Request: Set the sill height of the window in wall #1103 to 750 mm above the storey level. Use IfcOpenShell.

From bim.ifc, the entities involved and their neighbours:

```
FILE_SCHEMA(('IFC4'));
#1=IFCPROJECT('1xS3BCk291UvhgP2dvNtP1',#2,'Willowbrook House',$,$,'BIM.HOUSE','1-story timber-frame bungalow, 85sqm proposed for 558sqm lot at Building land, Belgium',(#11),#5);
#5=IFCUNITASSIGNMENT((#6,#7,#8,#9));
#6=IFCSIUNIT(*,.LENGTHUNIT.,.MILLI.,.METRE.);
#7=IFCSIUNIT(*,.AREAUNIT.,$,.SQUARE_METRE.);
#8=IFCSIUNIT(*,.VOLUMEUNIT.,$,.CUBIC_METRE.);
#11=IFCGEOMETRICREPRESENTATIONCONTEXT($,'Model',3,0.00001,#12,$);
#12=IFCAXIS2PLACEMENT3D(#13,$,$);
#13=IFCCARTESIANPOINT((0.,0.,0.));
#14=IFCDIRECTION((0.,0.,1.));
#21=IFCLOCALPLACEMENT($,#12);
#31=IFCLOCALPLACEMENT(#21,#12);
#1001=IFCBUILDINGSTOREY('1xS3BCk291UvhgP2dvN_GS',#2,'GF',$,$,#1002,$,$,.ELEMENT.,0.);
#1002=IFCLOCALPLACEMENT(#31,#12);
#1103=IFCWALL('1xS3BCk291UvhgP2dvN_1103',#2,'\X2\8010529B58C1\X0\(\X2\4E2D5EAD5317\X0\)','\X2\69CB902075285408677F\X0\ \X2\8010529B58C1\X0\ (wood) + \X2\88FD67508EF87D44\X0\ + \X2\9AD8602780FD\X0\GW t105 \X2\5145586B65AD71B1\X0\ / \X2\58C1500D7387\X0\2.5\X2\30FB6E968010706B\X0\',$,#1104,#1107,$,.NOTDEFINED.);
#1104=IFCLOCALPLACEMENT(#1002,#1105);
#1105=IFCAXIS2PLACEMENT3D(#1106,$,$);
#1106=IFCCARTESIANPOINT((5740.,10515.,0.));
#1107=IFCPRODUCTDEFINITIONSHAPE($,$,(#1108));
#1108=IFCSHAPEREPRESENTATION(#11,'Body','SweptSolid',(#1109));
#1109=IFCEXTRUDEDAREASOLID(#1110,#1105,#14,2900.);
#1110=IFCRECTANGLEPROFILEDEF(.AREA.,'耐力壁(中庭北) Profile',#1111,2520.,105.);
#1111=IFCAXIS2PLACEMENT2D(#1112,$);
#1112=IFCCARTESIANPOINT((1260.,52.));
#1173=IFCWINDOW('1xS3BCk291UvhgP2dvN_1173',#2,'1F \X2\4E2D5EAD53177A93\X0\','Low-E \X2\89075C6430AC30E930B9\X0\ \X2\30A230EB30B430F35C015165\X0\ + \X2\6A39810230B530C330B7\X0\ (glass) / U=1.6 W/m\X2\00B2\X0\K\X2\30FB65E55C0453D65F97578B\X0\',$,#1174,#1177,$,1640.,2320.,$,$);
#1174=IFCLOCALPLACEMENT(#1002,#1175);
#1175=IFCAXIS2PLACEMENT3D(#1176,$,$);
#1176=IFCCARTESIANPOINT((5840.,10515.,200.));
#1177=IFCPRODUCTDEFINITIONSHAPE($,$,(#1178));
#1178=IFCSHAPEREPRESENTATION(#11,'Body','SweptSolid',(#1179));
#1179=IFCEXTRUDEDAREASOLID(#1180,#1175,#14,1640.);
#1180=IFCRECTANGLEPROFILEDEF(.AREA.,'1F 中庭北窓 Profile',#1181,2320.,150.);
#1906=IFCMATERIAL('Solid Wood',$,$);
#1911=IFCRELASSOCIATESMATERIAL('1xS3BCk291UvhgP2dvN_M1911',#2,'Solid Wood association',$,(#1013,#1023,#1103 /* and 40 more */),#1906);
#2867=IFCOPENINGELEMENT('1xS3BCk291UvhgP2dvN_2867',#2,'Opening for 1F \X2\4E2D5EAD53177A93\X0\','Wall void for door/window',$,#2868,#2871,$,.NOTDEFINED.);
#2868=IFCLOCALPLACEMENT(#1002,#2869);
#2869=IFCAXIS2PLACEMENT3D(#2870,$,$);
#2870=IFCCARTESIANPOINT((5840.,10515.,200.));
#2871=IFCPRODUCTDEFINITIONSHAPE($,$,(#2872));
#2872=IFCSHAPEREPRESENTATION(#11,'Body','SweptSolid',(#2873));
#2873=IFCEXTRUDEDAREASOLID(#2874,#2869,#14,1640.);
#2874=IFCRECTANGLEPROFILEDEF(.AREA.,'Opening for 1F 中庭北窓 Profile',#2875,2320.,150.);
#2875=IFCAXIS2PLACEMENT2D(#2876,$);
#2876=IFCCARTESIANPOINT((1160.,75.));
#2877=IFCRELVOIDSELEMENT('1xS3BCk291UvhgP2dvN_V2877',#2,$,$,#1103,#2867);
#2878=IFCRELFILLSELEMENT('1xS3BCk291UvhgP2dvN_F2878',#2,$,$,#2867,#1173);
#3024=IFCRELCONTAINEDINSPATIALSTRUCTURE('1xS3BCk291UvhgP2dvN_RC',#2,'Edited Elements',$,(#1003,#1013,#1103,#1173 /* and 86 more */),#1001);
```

```python
import numpy as np
import ifcopenshell
import ifcopenshell.api.geometry
import ifcopenshell.geom
import ifcopenshell.util.element
import ifcopenshell.util.placement
import ifcopenshell.util.shape
import ifcopenshell.util.unit

model = ifcopenshell.open("bim.ifc")
unit_scale = ifcopenshell.util.unit.calculate_unit_scale(model)

window = model.by_guid("1xS3BCk291UvhgP2dvN_1173")
opening = window.FillsVoids[0].RelatingOpeningElement
storey = ifcopenshell.util.element.get_container(window, ifc_class="IfcBuildingStorey")
level = ifcopenshell.util.placement.get_local_placement(storey.ObjectPlacement)[2, 3]

# The opening's origin need not be at the sill, so measure its lowest point.
shape = ifcopenshell.geom.create_shape(ifcopenshell.geom.settings(), opening)
bottom = ifcopenshell.util.shape.get_shape_bottom_elevation(shape, shape.geometry) / unit_scale
dz = level + 0.75 / unit_scale - bottom

shift = np.array([0.0, 0.0, dz])
# The window is not placed relative to its opening, so move both.
for product in (opening, window):
    matrix = ifcopenshell.util.placement.get_local_placement(product.ObjectPlacement)
    matrix[:3, 3] += shift
    ifcopenshell.api.geometry.edit_object_placement(model, product=product, matrix=matrix, is_si=False)

print(f"moved by {dz * unit_scale:+.3f} m")

model.write("bim_rev.ifc")
```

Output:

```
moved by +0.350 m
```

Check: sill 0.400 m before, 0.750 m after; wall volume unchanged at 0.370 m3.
